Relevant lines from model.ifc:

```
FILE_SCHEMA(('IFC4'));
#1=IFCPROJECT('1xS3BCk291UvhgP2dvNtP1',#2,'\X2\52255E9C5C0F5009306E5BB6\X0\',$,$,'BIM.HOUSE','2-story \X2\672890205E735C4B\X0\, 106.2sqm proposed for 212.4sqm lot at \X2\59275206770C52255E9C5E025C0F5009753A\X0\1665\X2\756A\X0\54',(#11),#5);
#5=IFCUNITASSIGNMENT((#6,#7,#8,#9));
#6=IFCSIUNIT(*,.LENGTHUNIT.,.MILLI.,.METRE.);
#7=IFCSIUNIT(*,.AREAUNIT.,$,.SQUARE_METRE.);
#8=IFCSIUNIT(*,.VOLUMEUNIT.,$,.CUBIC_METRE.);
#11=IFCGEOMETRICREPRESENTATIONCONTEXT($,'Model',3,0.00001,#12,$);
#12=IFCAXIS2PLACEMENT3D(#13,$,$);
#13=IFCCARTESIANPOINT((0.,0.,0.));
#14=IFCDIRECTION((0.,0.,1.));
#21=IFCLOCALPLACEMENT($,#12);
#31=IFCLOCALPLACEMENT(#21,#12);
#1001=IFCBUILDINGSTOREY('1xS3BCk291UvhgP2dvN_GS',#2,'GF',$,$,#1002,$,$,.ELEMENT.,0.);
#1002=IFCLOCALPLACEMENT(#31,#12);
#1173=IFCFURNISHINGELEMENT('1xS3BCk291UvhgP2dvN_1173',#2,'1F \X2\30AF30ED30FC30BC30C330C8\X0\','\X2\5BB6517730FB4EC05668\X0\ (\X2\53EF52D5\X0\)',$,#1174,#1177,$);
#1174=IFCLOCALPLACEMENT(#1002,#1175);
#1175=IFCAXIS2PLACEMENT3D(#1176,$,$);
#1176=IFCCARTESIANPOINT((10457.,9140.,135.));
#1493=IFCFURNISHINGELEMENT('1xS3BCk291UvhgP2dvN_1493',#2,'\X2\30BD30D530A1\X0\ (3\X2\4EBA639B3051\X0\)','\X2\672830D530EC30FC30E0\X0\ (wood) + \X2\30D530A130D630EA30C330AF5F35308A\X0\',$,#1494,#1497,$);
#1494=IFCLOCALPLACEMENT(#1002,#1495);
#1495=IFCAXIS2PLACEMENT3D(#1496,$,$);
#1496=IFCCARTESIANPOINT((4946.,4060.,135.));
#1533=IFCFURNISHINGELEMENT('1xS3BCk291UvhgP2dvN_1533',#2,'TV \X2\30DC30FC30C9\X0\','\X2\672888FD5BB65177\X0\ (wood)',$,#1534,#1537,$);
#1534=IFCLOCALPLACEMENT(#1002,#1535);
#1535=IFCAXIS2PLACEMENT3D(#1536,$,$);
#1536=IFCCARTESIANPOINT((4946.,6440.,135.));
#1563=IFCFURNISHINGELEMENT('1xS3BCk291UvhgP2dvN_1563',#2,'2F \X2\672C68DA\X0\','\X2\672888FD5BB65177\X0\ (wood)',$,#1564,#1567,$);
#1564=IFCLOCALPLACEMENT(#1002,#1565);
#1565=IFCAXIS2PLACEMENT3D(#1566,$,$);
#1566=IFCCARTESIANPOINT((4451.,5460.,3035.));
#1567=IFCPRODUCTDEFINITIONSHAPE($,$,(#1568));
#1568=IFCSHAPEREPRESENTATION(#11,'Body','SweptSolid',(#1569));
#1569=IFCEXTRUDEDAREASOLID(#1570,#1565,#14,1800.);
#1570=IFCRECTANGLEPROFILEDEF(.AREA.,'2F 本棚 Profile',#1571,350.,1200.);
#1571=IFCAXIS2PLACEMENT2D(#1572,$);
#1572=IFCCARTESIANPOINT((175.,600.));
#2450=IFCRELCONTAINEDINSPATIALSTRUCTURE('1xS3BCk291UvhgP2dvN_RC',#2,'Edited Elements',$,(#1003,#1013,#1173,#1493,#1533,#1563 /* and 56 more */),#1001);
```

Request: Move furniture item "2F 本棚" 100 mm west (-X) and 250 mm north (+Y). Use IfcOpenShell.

```python
import ifcopenshell
import ifcopenshell.api.geometry
import ifcopenshell.util.placement
import ifcopenshell.util.unit

model = ifcopenshell.open("model.ifc")
unit_scale = ifcopenshell.util.unit.calculate_unit_scale(model)

item = model.by_guid("1xS3BCk291UvhgP2dvN_1563")
matrix = ifcopenshell.util.placement.get_local_placement(item.ObjectPlacement)
matrix[0, 3] -= 0.1 / unit_scale
matrix[1, 3] += 0.25 / unit_scale
ifcopenshell.api.geometry.edit_object_placement(model, product=item, matrix=matrix, is_si=False)

print(ifcopenshell.util.placement.get_local_placement(item.ObjectPlacement).round(3) + 0.0)

model.write("model-out.ifc")
```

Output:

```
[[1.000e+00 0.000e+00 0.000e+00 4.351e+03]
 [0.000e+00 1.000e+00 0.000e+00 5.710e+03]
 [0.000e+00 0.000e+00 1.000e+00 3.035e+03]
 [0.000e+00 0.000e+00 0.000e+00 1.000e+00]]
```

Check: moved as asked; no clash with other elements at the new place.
